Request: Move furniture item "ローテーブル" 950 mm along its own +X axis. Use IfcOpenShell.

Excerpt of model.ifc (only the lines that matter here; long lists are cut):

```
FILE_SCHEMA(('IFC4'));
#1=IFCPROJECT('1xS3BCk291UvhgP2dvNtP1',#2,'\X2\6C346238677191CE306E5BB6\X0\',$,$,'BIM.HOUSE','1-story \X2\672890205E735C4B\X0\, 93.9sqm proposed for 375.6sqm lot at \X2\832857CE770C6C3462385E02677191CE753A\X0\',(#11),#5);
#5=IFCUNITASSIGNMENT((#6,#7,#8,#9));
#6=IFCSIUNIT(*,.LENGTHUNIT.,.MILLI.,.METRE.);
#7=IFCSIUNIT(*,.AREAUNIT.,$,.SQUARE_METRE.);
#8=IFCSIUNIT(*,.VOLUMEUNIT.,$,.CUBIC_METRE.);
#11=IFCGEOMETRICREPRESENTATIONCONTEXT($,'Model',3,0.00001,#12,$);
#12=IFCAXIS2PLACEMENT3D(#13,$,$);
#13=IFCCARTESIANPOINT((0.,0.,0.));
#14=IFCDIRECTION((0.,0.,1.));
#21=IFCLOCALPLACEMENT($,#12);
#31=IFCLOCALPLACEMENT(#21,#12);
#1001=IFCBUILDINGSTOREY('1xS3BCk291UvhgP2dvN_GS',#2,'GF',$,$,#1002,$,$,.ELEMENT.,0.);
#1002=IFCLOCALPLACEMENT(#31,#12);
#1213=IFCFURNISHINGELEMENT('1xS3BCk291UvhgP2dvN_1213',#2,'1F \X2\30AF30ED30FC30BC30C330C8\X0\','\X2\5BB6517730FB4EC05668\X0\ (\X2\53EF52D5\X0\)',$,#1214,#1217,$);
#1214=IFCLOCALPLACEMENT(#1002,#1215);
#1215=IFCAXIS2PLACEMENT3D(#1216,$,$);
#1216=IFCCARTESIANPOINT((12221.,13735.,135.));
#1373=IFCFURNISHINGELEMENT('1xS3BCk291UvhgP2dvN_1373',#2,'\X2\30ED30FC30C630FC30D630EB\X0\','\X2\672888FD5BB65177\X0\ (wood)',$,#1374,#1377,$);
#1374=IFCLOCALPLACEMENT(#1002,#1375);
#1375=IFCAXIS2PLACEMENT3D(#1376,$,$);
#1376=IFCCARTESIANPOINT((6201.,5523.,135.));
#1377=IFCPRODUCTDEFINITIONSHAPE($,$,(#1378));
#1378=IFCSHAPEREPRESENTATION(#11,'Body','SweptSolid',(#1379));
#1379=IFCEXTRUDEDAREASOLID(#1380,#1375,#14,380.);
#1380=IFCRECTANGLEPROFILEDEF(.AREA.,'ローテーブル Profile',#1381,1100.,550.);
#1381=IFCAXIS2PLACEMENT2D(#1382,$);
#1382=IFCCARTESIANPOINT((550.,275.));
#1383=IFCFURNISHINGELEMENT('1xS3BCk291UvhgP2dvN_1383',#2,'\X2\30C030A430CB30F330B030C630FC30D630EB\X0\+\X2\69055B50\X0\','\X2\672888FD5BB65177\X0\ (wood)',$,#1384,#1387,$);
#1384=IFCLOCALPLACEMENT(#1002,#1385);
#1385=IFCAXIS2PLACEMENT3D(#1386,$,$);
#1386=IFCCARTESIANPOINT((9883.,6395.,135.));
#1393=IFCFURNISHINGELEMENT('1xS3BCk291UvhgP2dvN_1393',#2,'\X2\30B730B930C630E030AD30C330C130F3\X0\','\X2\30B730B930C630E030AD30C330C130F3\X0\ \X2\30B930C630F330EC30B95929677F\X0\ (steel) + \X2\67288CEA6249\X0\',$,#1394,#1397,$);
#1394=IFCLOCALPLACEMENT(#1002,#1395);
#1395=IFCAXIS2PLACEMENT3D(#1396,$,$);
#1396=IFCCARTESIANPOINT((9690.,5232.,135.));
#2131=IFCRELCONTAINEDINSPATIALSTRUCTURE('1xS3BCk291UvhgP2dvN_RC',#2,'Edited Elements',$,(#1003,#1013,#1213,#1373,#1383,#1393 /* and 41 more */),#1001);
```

```python
import ifcopenshell
import ifcopenshell.api.geometry
import ifcopenshell.util.placement
import ifcopenshell.util.unit

model = ifcopenshell.open("model.ifc")
unit_scale = ifcopenshell.util.unit.calculate_unit_scale(model)

item = model.by_guid("1xS3BCk291UvhgP2dvN_1373")
matrix = ifcopenshell.util.placement.get_local_placement(item.ObjectPlacement)
matrix[:3, 3] += matrix[:3, 0] * 0.95 / unit_scale
ifcopenshell.api.geometry.edit_object_placement(model, product=item, matrix=matrix, is_si=False)

print(ifcopenshell.util.placement.get_local_placement(item.ObjectPlacement).round(3) + 0.0)

model.write("model_v2.ifc")
```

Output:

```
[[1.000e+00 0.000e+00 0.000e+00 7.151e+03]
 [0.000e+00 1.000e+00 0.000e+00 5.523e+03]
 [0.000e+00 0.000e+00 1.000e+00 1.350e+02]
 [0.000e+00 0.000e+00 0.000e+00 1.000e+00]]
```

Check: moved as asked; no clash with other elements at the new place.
